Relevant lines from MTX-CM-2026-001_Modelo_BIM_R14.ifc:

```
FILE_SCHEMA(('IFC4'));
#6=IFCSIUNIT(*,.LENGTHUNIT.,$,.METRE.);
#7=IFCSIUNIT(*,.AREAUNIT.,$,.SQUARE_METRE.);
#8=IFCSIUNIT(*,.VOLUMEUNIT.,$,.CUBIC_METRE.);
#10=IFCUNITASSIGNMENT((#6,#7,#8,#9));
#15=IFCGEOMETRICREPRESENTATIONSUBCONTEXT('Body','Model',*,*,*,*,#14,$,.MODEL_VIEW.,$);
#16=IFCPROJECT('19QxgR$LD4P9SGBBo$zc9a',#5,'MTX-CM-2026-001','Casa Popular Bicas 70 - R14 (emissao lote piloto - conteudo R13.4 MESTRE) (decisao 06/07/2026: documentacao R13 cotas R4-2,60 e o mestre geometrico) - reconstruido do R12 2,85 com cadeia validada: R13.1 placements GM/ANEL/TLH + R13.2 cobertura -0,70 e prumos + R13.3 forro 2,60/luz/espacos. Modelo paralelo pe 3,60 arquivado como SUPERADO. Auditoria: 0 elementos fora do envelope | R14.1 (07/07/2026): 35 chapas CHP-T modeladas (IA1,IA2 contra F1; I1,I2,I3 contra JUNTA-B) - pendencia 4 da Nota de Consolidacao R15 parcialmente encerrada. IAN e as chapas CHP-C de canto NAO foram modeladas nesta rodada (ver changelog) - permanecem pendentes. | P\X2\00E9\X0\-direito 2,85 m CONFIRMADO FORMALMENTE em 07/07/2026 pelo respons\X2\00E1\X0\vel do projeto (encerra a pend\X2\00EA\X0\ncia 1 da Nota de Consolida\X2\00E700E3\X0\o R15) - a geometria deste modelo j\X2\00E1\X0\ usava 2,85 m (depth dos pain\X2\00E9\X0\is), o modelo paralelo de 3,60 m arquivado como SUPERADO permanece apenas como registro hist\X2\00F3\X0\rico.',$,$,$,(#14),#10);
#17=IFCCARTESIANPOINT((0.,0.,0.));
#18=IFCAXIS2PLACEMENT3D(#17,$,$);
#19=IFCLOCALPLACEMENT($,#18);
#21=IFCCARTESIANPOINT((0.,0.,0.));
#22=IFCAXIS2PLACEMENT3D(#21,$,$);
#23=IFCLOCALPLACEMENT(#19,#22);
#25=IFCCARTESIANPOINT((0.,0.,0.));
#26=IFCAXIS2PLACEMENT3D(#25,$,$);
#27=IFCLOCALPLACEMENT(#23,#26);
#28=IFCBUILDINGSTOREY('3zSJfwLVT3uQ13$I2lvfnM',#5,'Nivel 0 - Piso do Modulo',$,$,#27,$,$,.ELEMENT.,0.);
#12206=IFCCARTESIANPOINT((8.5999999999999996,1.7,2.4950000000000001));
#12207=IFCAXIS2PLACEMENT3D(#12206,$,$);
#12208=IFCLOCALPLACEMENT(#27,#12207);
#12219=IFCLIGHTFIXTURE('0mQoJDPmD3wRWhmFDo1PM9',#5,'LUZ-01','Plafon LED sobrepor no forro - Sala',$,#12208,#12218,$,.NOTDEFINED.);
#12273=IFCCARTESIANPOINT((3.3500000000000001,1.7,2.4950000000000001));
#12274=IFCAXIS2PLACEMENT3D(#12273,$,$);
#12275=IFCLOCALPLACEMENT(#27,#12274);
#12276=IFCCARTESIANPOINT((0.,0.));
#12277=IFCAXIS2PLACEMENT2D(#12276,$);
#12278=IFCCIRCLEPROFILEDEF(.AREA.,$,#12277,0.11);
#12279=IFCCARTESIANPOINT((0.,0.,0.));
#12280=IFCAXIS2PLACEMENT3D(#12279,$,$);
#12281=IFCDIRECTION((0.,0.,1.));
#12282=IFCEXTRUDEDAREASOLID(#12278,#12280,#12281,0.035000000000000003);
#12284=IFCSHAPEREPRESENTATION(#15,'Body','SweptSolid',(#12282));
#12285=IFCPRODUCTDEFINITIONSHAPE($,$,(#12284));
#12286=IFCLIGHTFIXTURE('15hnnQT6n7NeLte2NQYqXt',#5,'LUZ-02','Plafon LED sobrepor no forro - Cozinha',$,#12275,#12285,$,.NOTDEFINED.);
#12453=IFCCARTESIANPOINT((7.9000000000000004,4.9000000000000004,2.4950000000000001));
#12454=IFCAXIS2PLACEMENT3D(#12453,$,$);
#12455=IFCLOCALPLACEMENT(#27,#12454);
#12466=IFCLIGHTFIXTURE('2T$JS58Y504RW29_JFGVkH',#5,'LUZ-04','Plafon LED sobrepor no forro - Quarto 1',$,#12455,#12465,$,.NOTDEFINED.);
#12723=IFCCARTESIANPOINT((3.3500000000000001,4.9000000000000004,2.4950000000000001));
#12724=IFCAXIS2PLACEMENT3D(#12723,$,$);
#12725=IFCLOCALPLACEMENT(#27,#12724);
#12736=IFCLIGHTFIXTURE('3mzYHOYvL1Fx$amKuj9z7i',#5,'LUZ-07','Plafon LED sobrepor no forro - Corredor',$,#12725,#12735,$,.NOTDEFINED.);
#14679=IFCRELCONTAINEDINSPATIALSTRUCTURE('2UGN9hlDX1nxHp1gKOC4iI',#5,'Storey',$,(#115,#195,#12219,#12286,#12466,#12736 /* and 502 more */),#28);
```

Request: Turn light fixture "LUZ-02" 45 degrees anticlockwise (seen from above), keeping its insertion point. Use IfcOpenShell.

```python
import ifcopenshell
import ifcopenshell.api.geometry
import ifcopenshell.util.placement

model = ifcopenshell.open("MTX-CM-2026-001_Modelo_BIM_R14.ifc")

item = model.by_guid("15hnnQT6n7NeLte2NQYqXt")
matrix = ifcopenshell.util.placement.get_local_placement(item.ObjectPlacement)
matrix = matrix @ ifcopenshell.util.placement.rotation(45, "Z")
ifcopenshell.api.geometry.edit_object_placement(model, product=item, matrix=matrix, is_si=False)

print(ifcopenshell.util.placement.get_local_placement(item.ObjectPlacement).round(3) + 0.0)

model.write("MTX-CM-2026-001_Modelo_BIM_R14-out.ifc")
```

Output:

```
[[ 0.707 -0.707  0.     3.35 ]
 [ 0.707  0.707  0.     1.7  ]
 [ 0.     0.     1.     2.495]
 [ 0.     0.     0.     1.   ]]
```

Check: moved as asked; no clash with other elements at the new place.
